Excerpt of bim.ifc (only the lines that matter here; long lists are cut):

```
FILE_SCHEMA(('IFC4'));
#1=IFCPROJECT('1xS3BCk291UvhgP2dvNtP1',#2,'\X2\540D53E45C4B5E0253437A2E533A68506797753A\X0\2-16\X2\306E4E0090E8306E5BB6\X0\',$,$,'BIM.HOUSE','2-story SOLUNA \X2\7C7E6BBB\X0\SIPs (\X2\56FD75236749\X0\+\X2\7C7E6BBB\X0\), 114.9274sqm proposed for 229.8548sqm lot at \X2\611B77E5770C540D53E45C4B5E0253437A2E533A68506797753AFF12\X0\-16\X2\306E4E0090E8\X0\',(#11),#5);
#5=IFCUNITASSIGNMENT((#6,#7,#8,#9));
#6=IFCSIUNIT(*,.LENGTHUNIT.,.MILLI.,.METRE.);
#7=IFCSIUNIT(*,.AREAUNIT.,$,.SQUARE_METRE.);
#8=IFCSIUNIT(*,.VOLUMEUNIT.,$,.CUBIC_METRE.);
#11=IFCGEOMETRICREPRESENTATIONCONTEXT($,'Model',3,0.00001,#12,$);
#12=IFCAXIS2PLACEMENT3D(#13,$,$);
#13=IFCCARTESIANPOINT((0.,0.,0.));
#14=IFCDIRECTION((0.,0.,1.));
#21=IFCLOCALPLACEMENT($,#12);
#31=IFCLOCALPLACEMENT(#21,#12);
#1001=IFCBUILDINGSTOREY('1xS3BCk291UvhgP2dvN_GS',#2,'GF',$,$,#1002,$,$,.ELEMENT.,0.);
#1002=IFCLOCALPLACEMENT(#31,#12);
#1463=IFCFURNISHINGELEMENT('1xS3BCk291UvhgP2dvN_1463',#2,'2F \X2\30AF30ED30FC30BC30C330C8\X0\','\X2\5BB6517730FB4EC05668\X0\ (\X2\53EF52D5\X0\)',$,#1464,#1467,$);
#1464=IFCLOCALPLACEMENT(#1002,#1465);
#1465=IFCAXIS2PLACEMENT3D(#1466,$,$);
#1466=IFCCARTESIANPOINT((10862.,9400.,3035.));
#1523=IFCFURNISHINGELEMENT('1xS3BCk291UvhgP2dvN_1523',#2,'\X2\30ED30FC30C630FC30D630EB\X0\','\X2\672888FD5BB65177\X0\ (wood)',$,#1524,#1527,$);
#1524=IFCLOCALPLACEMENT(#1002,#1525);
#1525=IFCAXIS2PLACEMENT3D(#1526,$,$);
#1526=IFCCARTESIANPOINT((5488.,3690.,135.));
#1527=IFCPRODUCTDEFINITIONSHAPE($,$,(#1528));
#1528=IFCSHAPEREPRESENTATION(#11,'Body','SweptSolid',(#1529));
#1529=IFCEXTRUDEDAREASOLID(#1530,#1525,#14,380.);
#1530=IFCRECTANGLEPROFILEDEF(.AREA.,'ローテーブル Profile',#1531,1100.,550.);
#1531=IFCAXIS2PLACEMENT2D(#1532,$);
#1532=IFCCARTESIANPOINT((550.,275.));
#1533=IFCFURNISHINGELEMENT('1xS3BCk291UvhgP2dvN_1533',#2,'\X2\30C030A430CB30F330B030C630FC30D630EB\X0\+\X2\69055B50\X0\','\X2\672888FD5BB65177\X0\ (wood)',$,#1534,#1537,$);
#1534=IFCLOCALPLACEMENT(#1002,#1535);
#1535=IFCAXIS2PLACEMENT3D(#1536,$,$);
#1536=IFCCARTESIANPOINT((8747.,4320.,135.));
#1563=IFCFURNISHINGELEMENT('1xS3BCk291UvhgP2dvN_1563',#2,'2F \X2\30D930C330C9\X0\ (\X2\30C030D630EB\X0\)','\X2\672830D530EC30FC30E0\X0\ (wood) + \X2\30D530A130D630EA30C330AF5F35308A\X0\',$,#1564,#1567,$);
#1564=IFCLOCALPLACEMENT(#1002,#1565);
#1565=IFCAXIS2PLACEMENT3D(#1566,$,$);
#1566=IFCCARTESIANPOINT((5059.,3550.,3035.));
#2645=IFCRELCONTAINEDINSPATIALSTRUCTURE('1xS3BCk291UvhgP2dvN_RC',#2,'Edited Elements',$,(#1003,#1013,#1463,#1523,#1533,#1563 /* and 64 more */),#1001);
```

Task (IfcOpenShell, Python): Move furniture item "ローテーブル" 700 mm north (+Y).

```python
import ifcopenshell
import ifcopenshell.api.geometry
import ifcopenshell.util.placement
import ifcopenshell.util.unit

model = ifcopenshell.open("bim.ifc")
unit_scale = ifcopenshell.util.unit.calculate_unit_scale(model)

item = model.by_guid("1xS3BCk291UvhgP2dvN_1523")
matrix = ifcopenshell.util.placement.get_local_placement(item.ObjectPlacement)
matrix[1, 3] += 0.7 / unit_scale
ifcopenshell.api.geometry.edit_object_placement(model, product=item, matrix=matrix, is_si=False)

print(ifcopenshell.util.placement.get_local_placement(item.ObjectPlacement).round(3) + 0.0)

model.write("bim-out.ifc")
```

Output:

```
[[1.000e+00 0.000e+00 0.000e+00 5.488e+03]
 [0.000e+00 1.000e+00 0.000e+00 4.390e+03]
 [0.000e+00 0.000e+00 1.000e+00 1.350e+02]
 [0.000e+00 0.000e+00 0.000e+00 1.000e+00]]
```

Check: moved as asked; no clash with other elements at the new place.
